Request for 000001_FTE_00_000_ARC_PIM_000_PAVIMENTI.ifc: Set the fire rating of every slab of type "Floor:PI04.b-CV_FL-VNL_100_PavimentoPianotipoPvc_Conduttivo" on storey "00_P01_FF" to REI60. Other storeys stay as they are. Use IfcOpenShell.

First a look at what the model holds.

```python
import ifcopenshell
import ifcopenshell.util.element

model = ifcopenshell.open("000001_FTE_00_000_ARC_PIM_000_PAVIMENTI.ifc")
print(model.schema)
storey = next(s for s in model.by_type("IfcBuildingStorey") if s.Name == "00_P01_FF")
slabs = [e for e in ifcopenshell.util.element.get_decomposition(storey) if e.is_a("IfcSlab")]
seen = {}
for e in slabs:
    element_type = ifcopenshell.util.element.get_type(e)
    key = (element_type.Name if element_type != e and element_type else None, ifcopenshell.util.element.get_pset(e, "Pset_SlabCommon", "FireRating"))
    seen[key] = seen.get(key, 0) + 1
for (name, value), count in sorted(seen.items(), key=str):
    print(count, "x", name, "|", value)
```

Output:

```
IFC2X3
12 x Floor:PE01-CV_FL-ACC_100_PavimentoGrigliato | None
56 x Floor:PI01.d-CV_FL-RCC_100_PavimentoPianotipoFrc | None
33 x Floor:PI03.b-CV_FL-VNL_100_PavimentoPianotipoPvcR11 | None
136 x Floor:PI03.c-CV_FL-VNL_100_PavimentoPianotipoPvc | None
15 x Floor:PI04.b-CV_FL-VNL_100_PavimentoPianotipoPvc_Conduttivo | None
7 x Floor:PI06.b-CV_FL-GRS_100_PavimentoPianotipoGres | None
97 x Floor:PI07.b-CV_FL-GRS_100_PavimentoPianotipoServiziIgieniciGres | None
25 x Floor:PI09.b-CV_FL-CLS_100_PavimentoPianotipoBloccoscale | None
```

```python
import ifcopenshell
import ifcopenshell.api.pset
import ifcopenshell.util.element

model = ifcopenshell.open("000001_FTE_00_000_ARC_PIM_000_PAVIMENTI.ifc")

storey = next(s for s in model.by_type("IfcBuildingStorey") if s.Name == "00_P01_FF")
slabs = [e for e in ifcopenshell.util.element.get_decomposition(storey) if e.is_a("IfcSlab")]

count = 0
for e in slabs:
    element_type = ifcopenshell.util.element.get_type(e)
    if element_type in (None, e) or element_type.Name != "Floor:PI04.b-CV_FL-VNL_100_PavimentoPianotipoPvc_Conduttivo":
        continue
    # add_pset returns the element's existing set when there is one.
    pset = ifcopenshell.api.pset.add_pset(model, product=e, name="Pset_SlabCommon")
    ifcopenshell.api.pset.edit_pset(model, pset=pset, properties={"FireRating": "REI60"})
    count += 1

print(count, "slabs updated")

model.write("000001_FTE_00_000_ARC_PIM_000_PAVIMENTI-out.ifc")
```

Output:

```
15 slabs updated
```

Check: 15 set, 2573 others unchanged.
